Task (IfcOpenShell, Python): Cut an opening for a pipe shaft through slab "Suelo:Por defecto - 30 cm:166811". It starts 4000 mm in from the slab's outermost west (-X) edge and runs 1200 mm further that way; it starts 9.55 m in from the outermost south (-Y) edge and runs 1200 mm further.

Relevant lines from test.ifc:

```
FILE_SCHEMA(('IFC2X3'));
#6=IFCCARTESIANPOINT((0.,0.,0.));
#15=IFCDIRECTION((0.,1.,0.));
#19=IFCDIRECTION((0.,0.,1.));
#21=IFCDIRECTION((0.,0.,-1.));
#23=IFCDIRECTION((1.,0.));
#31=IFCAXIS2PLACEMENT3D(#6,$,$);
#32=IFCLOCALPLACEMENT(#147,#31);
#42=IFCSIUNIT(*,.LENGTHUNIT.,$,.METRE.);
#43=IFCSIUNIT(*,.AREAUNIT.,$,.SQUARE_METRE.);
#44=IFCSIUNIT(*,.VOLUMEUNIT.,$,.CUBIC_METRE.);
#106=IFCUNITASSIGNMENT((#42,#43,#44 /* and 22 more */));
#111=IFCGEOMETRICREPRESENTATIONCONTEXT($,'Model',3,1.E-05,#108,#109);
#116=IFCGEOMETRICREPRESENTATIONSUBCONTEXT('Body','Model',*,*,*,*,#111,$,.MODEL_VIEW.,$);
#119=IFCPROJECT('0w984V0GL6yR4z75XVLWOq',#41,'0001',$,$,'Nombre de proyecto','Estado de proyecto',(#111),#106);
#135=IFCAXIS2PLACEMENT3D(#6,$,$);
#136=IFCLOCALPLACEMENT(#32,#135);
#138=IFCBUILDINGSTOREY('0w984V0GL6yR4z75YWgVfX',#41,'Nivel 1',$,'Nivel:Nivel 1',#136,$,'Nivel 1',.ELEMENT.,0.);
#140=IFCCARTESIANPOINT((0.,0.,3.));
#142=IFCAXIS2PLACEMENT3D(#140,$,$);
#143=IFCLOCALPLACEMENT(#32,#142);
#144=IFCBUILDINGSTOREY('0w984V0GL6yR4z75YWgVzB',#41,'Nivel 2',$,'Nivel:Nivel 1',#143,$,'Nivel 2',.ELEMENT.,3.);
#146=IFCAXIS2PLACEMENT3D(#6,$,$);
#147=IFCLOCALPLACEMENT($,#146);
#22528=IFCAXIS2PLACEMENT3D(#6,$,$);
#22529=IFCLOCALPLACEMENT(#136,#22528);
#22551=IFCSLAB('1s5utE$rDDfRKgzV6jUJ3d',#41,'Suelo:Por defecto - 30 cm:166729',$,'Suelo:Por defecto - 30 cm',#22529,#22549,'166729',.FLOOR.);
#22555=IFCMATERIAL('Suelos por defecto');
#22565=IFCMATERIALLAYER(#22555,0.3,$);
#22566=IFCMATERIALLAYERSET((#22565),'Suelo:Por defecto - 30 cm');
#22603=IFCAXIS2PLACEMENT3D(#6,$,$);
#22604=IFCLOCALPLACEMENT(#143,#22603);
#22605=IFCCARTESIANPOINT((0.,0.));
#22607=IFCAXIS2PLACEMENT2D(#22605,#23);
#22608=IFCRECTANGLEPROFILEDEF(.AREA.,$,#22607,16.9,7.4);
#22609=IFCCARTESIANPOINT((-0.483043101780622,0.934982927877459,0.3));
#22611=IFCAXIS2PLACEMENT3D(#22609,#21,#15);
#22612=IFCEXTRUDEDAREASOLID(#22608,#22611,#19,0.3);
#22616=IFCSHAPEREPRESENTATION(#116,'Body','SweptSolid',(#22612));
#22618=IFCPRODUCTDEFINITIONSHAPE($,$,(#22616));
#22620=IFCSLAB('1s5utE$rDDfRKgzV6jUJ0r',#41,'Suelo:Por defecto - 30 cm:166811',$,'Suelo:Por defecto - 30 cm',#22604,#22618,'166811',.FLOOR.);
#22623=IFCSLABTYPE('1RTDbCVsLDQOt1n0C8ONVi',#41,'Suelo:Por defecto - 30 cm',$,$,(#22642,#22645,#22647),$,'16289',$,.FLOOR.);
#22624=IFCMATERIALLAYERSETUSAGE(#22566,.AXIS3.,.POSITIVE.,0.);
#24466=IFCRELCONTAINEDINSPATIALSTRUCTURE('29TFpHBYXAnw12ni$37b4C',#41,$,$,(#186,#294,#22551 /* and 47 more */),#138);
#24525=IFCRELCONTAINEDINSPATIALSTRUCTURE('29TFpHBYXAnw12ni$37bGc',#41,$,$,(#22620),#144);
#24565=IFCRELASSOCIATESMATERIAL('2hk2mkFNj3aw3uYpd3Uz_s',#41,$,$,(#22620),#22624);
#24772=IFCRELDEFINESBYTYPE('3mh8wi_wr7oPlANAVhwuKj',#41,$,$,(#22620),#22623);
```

```python
import numpy as np
import ifcopenshell
import ifcopenshell.api.feature
import ifcopenshell.api.geometry
import ifcopenshell.api.root
import ifcopenshell.geom
import ifcopenshell.util.placement
import ifcopenshell.util.representation
import ifcopenshell.util.shape
import ifcopenshell.util.unit

model = ifcopenshell.open("test.ifc")
unit_scale = ifcopenshell.util.unit.calculate_unit_scale(model)
settings = ifcopenshell.geom.settings()


def volume(element):
    """Net volume in cubic metres, openings subtracted."""
    shape = ifcopenshell.geom.create_shape(settings, element)
    return ifcopenshell.util.shape.get_volume(shape.geometry)


slab = model.by_guid("1s5utE$rDDfRKgzV6jUJ0r")
before = volume(slab)

# Extent in the slab's own axes, in metres. The edges named are its -X and -Y sides.
slab_shape = ifcopenshell.geom.create_shape(settings, slab)
vertices = ifcopenshell.util.shape.get_vertices(slab_shape.geometry)
x_min, y_min, bottom = vertices.min(axis=0)
top = vertices[:, 2].max()

opening = ifcopenshell.api.root.create_entity(model, ifc_class="IfcOpeningElement", name="Pipe shaft opening")
context = ifcopenshell.util.representation.get_context(model, "Model", "Body", "MODEL_VIEW")
width, depth = 1.2, 1.2
outline = [(0.0, 0.0), (width, 0.0), (width, depth), (0.0, depth), (0.0, 0.0)]
# Overshoot both faces by 50 mm so the cut is clean.
shape = ifcopenshell.api.geometry.add_slab_representation(
    model, context=context, depth=top - bottom + 0.1, polyline=outline
)
ifcopenshell.api.geometry.assign_representation(model, product=opening, representation=shape)

matrix = ifcopenshell.util.placement.get_local_placement(slab.ObjectPlacement)
matrix[:, 3] = matrix @ np.append(np.array([x_min + 4, y_min + 9.55, bottom - 0.05]) / unit_scale, 1.0)
ifcopenshell.api.geometry.edit_object_placement(model, product=opening, matrix=matrix, is_si=False)
ifcopenshell.api.feature.add_feature(model, feature=opening, element=slab)

after = volume(slab)

print(f"slab volume {before:.3f} -> {after:.3f} m3")

model.write("test_edited.ifc")
```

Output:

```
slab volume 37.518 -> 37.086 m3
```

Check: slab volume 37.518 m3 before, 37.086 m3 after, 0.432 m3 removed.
